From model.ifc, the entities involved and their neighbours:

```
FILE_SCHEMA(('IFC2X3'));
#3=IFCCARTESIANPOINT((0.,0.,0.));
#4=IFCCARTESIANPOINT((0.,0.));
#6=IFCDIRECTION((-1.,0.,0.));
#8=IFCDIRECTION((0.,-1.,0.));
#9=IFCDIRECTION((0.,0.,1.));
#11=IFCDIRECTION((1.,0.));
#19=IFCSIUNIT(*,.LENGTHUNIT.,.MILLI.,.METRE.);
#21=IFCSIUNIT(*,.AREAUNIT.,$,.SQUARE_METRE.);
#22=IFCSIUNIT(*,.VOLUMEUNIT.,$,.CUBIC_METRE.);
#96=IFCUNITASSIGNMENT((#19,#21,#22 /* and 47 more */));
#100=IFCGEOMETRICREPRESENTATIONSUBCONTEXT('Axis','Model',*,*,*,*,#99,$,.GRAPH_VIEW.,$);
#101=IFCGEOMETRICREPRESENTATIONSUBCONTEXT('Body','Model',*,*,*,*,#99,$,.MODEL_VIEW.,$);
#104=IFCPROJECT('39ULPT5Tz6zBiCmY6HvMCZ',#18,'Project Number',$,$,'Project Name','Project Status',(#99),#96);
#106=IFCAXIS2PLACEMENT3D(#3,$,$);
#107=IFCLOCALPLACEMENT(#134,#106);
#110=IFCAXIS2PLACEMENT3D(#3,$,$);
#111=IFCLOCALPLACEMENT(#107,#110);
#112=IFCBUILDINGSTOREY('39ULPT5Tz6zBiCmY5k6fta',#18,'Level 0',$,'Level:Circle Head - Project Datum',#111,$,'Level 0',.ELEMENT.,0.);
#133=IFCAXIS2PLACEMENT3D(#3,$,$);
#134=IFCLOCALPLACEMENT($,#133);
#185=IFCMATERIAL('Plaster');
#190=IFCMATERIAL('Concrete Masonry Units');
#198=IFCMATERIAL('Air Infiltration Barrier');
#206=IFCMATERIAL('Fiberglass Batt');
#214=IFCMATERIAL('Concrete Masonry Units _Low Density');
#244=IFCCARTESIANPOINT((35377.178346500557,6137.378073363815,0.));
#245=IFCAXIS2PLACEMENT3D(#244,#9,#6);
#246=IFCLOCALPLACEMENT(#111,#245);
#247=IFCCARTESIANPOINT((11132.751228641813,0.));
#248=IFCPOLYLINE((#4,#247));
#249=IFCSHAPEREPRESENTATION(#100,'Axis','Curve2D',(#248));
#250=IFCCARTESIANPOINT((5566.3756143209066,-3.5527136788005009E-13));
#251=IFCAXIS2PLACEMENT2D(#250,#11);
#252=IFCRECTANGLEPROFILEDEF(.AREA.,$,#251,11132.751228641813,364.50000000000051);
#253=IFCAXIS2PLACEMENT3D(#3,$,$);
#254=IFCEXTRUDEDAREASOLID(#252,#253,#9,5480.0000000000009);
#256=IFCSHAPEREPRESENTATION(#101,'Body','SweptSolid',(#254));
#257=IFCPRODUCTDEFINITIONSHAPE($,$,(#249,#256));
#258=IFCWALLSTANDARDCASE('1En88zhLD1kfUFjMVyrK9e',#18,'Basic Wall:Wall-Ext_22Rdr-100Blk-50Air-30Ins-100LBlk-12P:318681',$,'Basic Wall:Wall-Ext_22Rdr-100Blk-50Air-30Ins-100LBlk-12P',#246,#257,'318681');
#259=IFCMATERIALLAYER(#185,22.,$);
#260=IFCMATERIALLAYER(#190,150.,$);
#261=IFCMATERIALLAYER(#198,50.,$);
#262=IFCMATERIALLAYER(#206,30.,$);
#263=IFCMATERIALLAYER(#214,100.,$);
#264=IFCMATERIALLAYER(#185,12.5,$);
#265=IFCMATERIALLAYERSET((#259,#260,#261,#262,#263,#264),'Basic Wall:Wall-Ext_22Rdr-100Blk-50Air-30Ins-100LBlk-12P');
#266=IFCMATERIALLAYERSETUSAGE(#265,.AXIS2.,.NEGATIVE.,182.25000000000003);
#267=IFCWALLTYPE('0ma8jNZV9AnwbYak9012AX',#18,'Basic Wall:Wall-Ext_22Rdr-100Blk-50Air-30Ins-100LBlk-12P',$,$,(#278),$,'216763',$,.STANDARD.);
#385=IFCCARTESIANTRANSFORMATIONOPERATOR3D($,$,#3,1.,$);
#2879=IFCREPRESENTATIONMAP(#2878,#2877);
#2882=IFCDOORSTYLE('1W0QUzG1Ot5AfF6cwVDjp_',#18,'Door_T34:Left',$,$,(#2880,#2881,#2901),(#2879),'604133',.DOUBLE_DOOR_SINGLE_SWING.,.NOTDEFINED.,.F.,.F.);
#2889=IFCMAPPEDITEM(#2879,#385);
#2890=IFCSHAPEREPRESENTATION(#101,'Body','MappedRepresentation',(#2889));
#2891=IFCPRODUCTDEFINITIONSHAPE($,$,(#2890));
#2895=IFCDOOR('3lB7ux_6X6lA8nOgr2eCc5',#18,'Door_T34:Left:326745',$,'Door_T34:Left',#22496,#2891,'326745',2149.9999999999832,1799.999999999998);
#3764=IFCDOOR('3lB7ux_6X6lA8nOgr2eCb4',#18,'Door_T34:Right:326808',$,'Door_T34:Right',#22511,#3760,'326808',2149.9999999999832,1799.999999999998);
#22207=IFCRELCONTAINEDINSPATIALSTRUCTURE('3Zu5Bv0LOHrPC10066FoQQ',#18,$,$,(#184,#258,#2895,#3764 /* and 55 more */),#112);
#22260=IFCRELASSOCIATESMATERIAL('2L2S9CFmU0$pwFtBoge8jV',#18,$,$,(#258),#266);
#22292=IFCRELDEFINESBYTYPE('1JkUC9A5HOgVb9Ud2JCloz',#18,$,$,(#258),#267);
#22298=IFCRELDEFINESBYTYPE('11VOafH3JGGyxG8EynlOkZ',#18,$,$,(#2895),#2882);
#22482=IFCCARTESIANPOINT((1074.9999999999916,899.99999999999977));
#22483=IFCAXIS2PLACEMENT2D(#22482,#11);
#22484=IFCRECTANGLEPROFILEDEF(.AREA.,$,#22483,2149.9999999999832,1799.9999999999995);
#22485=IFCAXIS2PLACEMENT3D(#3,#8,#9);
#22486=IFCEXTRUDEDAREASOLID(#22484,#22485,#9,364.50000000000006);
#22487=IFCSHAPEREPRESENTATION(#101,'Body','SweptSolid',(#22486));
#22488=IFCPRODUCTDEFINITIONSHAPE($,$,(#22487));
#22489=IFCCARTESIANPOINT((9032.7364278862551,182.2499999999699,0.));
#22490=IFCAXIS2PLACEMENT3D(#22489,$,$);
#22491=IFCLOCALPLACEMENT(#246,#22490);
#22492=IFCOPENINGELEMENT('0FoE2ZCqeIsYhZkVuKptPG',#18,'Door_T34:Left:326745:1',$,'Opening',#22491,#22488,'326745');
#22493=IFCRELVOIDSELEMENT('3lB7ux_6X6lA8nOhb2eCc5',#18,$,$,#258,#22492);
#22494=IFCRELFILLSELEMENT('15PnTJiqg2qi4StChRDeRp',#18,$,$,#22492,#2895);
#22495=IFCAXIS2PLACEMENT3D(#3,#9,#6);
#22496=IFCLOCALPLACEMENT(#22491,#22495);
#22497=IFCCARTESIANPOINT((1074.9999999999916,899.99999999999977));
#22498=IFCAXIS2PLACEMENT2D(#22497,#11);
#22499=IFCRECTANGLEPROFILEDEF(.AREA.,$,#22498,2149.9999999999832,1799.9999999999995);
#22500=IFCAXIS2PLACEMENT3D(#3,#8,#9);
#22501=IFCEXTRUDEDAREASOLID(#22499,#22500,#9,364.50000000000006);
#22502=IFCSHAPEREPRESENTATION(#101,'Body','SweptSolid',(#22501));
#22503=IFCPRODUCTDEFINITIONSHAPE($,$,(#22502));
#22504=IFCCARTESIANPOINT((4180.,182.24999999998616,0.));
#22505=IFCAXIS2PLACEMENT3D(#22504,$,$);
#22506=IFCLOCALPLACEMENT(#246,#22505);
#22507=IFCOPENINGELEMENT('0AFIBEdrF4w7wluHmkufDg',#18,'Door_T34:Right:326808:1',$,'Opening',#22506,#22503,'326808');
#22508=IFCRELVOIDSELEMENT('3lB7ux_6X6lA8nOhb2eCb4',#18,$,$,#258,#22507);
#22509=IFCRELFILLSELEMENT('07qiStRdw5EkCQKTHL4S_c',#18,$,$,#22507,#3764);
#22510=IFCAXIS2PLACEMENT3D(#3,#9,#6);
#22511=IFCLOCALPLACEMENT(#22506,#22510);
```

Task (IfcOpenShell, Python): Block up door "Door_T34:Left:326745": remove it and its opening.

```python
import ifcopenshell
import ifcopenshell.api.feature
import ifcopenshell.api.root
import ifcopenshell.geom
import ifcopenshell.util.shape

model = ifcopenshell.open("model.ifc")
settings = ifcopenshell.geom.settings()


def volume(element):
    """Net volume in cubic metres, openings subtracted."""
    shape = ifcopenshell.geom.create_shape(settings, element)
    return ifcopenshell.util.shape.get_volume(shape.geometry)


door = model.by_guid("3lB7ux_6X6lA8nOgr2eCc5")
opening = door.FillsVoids[0].RelatingOpeningElement
wall = opening.VoidsElements[0].RelatingBuildingElement
before = volume(wall)

ifcopenshell.api.root.remove_product(model, product=door)
ifcopenshell.api.feature.remove_feature(model, feature=opening)

after = volume(wall)

print(f"wall volume {before:.3f} -> {after:.3f} m3")

model.write("model_v2.ifc")
```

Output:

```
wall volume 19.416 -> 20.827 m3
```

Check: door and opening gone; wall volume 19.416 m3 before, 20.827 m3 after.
